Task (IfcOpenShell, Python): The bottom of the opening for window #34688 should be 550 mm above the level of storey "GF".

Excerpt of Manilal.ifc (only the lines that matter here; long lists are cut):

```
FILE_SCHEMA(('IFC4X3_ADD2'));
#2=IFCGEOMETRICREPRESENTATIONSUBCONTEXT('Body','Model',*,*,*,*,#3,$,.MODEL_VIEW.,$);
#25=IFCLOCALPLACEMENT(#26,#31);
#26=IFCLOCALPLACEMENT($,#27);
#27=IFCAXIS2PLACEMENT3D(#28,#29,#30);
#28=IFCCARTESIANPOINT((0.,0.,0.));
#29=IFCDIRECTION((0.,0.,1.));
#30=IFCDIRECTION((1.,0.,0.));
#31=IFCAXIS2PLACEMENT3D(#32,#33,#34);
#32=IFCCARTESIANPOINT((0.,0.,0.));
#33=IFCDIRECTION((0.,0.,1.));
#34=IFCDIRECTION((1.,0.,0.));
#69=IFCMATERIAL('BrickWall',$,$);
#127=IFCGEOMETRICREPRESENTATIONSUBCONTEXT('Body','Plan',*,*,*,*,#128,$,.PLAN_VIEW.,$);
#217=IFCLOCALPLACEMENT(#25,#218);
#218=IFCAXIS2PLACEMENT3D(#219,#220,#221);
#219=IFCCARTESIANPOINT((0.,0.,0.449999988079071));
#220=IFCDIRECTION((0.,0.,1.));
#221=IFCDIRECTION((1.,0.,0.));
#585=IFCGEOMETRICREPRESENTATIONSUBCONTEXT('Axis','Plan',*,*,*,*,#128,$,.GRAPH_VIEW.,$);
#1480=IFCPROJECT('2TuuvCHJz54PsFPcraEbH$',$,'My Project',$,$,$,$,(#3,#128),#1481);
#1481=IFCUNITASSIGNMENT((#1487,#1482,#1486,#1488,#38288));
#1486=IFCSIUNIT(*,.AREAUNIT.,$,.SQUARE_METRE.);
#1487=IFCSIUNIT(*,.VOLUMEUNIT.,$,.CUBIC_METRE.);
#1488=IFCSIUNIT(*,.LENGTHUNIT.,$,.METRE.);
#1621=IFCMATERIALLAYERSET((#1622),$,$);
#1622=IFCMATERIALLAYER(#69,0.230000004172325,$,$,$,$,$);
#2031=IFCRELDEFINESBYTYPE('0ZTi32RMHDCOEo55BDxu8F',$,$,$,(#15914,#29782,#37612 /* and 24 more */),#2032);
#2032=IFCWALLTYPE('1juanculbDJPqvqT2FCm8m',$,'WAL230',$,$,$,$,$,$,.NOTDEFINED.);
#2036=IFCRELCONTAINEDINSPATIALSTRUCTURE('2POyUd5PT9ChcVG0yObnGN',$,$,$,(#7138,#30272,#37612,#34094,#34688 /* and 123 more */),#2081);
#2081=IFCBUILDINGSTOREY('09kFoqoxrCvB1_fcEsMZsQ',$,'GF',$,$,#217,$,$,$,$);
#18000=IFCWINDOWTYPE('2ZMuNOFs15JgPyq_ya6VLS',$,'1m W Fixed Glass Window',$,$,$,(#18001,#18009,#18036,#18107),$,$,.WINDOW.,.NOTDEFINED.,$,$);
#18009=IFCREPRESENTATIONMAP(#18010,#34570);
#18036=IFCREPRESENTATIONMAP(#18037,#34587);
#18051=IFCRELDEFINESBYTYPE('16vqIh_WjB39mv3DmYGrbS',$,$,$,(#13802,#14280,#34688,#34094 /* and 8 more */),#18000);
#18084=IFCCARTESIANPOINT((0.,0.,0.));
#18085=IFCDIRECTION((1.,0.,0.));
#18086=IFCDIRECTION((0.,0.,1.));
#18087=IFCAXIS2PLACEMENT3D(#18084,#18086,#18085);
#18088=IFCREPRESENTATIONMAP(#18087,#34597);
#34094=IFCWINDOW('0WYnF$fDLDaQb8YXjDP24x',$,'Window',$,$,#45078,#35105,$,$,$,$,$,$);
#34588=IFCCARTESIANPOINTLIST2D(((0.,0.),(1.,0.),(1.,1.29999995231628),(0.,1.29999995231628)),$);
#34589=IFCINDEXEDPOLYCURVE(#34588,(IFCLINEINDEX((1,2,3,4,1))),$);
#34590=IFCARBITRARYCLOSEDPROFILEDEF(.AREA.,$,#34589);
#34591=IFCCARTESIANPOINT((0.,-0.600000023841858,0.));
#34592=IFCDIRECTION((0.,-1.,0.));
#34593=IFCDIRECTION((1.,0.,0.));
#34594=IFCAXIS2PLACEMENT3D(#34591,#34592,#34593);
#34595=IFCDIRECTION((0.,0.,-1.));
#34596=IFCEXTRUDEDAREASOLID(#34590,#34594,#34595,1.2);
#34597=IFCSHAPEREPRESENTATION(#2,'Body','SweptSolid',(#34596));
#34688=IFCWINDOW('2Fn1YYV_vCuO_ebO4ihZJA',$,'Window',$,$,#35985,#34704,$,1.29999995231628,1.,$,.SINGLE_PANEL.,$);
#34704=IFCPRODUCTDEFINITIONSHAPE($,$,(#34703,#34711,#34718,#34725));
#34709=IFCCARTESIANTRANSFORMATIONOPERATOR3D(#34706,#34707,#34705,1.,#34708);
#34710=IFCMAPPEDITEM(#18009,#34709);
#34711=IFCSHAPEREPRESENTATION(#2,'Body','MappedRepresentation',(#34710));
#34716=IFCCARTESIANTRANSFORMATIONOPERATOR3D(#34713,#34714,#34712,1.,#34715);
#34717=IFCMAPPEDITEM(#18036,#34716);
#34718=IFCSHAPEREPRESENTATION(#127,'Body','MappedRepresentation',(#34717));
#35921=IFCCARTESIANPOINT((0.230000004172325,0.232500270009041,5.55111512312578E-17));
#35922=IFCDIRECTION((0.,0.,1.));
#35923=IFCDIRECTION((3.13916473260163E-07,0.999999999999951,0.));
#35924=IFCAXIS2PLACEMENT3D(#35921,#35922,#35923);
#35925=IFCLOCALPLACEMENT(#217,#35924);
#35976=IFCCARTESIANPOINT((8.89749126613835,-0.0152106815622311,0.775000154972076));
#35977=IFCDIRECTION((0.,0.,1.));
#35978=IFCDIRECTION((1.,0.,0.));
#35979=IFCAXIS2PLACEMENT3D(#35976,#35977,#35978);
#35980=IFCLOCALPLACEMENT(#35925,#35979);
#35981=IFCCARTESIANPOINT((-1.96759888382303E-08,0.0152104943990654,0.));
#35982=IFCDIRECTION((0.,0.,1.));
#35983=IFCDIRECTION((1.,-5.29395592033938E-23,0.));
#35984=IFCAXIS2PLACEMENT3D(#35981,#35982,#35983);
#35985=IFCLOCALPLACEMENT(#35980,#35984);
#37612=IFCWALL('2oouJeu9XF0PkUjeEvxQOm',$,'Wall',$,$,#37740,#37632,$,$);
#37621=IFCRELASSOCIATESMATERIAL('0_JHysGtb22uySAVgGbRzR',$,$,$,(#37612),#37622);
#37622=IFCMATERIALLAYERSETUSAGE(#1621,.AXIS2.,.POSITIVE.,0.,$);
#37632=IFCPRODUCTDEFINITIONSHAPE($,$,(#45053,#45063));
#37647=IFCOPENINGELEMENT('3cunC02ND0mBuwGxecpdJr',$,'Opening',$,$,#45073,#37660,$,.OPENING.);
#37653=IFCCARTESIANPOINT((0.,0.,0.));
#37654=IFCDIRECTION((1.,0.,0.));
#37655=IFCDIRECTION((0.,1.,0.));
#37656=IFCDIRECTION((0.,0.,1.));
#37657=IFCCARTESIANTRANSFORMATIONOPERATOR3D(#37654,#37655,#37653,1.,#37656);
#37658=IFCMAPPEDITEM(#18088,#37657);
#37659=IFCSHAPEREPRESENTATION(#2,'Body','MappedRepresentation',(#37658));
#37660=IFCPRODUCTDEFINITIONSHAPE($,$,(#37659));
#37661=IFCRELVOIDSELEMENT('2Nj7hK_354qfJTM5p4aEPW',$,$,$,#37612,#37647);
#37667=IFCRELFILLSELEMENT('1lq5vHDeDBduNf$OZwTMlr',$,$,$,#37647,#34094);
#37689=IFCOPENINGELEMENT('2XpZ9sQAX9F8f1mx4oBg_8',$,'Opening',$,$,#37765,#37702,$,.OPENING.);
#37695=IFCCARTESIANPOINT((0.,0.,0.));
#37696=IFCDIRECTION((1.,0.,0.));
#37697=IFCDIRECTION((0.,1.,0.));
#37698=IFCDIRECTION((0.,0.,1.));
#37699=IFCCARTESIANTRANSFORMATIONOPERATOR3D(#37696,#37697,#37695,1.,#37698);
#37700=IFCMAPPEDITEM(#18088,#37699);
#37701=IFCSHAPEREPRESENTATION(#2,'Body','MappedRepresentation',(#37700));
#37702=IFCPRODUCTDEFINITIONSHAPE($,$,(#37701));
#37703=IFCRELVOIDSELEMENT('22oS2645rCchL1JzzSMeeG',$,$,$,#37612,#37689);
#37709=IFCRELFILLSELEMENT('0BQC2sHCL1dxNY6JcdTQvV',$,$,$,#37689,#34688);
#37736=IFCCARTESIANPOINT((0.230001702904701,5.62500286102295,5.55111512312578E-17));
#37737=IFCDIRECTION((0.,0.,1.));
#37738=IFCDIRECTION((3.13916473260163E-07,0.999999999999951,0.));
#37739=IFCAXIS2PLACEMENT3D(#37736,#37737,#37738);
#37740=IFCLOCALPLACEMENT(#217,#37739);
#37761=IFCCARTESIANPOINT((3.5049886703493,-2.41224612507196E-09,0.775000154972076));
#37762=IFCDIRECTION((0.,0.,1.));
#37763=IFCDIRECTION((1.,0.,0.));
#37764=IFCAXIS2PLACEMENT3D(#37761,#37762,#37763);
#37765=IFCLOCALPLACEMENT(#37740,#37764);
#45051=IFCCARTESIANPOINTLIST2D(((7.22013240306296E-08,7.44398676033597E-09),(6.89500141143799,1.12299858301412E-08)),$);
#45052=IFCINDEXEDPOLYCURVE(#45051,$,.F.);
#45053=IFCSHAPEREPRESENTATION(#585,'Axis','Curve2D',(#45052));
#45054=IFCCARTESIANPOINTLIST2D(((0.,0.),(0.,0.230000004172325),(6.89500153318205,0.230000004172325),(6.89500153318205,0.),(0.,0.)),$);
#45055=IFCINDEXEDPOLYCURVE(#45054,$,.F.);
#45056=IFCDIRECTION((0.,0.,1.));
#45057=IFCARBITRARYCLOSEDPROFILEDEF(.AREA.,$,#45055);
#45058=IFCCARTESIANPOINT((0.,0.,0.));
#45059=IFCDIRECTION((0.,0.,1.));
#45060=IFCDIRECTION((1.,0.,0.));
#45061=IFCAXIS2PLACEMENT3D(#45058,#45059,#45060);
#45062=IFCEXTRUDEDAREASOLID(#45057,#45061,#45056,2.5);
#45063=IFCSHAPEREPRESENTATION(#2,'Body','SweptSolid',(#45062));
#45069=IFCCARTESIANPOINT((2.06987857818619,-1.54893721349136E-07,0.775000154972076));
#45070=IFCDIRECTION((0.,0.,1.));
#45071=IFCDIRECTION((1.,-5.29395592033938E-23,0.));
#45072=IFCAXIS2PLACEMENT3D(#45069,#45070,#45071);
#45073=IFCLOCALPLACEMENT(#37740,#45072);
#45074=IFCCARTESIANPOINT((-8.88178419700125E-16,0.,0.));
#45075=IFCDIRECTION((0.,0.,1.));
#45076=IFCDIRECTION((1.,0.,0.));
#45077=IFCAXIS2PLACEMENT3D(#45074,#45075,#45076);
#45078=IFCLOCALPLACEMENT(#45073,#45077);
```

```python
import numpy as np
import ifcopenshell
import ifcopenshell.api.geometry
import ifcopenshell.geom
import ifcopenshell.util.element
import ifcopenshell.util.placement
import ifcopenshell.util.shape
import ifcopenshell.util.unit

model = ifcopenshell.open("Manilal.ifc")
unit_scale = ifcopenshell.util.unit.calculate_unit_scale(model)

window = model.by_guid("2Fn1YYV_vCuO_ebO4ihZJA")
opening = window.FillsVoids[0].RelatingOpeningElement
storey = ifcopenshell.util.element.get_container(window, ifc_class="IfcBuildingStorey")
level = ifcopenshell.util.placement.get_local_placement(storey.ObjectPlacement)[2, 3]

# The opening's origin need not be at the sill, so measure its lowest point.
shape = ifcopenshell.geom.create_shape(ifcopenshell.geom.settings(), opening)
bottom = ifcopenshell.util.shape.get_shape_bottom_elevation(shape, shape.geometry) / unit_scale
dz = level + 0.55 / unit_scale - bottom

shift = np.array([0.0, 0.0, dz])
# The window is not placed relative to its opening, so move both.
for product in (opening, window):
    matrix = ifcopenshell.util.placement.get_local_placement(product.ObjectPlacement)
    matrix[:3, 3] += shift
    ifcopenshell.api.geometry.edit_object_placement(model, product=product, matrix=matrix, is_si=False)

print(f"moved by {dz * unit_scale:+.3f} m")

model.write("Manilal_v2.ifc")
```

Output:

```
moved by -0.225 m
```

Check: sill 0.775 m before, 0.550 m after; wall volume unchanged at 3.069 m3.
